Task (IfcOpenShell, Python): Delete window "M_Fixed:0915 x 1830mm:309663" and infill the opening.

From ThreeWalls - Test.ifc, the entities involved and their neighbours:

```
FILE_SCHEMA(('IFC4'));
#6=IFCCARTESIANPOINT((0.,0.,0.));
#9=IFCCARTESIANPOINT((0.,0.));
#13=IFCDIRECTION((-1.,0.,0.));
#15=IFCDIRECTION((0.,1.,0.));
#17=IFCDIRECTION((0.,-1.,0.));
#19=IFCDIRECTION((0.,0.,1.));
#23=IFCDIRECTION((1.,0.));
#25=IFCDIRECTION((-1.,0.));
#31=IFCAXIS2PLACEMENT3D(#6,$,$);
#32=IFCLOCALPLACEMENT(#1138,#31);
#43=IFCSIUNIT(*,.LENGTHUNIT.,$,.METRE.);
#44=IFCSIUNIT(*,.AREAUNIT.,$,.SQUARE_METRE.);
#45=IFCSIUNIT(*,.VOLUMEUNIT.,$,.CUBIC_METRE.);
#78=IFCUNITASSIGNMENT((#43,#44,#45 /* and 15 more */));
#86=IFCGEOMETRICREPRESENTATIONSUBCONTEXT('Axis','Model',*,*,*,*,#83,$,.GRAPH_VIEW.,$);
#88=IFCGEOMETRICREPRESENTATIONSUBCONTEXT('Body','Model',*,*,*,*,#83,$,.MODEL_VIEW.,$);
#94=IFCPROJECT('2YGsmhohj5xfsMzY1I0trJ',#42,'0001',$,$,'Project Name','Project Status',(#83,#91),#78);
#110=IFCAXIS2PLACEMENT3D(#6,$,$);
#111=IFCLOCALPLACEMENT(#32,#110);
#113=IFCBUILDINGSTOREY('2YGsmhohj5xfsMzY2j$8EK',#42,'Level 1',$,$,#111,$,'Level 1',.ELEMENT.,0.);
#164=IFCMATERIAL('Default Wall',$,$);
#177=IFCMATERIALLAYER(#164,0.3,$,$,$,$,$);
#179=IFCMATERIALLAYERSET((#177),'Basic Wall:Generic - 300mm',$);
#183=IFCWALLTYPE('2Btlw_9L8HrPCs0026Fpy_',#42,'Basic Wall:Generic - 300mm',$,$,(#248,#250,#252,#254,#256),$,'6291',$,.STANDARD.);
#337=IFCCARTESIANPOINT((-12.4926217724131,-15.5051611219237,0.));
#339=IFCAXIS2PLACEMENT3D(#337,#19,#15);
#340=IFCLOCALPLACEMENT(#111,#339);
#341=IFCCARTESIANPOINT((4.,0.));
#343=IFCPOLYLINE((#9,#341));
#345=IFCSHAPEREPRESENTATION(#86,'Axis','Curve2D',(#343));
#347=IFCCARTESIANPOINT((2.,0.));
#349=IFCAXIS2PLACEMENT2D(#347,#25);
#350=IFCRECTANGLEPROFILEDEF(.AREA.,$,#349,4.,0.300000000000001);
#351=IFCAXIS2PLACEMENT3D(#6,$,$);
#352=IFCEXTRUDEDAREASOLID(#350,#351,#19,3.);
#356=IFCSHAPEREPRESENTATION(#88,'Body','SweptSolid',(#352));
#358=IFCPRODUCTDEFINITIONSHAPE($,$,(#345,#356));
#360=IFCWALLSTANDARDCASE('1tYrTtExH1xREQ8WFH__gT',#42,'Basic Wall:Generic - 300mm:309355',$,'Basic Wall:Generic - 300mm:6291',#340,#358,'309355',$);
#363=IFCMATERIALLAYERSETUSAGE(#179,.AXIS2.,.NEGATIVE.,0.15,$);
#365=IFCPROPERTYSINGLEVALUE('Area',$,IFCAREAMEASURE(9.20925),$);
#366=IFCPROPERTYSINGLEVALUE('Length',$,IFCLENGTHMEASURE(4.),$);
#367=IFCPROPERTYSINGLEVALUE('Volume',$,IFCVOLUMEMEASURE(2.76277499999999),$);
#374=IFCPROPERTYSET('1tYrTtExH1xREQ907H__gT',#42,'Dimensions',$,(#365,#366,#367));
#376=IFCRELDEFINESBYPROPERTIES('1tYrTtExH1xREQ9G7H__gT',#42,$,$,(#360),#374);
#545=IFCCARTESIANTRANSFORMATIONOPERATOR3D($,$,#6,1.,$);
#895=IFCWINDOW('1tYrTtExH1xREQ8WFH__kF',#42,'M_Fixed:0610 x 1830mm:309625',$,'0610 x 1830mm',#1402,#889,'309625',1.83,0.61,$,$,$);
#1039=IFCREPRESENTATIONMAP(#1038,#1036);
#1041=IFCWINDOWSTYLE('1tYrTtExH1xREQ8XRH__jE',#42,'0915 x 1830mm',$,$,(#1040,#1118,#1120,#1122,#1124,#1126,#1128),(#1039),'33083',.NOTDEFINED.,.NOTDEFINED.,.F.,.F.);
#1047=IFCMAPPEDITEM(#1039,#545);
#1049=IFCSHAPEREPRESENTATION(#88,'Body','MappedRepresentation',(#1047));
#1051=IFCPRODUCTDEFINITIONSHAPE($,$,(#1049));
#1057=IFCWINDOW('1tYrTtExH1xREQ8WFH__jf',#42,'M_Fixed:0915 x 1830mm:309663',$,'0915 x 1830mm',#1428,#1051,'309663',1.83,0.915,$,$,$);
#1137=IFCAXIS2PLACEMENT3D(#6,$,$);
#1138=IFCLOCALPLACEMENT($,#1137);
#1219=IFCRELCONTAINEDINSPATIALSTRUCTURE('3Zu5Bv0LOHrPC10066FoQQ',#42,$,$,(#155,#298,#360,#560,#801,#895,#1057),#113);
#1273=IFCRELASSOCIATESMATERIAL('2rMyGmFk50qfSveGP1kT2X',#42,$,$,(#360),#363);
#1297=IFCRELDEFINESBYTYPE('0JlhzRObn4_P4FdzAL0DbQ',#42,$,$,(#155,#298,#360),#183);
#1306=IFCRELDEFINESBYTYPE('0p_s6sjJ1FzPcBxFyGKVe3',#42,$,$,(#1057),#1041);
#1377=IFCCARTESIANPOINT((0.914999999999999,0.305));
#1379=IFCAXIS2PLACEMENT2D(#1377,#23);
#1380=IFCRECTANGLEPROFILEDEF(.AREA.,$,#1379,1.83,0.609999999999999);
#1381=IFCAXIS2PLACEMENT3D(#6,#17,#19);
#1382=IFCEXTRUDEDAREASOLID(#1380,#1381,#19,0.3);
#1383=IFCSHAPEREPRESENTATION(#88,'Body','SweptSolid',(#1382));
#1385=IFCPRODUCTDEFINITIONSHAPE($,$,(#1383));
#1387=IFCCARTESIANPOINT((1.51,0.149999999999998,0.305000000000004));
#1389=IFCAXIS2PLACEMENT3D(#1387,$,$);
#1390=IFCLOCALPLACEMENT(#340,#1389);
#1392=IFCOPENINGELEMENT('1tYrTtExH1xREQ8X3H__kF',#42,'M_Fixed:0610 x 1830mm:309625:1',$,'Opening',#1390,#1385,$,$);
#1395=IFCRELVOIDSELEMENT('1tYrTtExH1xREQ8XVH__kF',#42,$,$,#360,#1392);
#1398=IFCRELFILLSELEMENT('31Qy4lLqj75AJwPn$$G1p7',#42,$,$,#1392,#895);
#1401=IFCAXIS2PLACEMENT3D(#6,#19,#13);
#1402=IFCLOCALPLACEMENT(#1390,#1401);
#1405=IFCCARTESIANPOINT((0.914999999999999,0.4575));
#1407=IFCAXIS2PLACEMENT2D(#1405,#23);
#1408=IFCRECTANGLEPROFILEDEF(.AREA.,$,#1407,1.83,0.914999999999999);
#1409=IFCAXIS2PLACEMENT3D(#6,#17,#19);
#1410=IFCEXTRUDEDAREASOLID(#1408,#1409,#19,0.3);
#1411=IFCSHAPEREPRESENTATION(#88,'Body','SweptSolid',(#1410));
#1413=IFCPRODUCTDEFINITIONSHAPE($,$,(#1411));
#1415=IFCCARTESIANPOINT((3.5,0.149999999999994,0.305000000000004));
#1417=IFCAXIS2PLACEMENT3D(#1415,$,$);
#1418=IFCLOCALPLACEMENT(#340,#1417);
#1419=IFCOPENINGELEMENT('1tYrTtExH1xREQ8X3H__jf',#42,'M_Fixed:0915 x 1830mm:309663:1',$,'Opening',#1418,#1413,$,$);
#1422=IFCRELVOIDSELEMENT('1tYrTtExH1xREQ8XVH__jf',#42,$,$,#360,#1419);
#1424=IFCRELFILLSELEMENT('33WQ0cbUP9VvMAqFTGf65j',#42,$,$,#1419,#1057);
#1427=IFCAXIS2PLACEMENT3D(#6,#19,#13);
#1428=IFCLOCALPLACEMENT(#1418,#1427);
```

```python
import ifcopenshell
import ifcopenshell.api.feature
import ifcopenshell.api.pset
import ifcopenshell.api.root
import ifcopenshell.geom
import ifcopenshell.util.element
import ifcopenshell.util.shape
import ifcopenshell.util.unit

model = ifcopenshell.open("ThreeWalls - Test.ifc")
area_scale = ifcopenshell.util.unit.calculate_unit_scale(model, "AREAUNIT")
volume_scale = ifcopenshell.util.unit.calculate_unit_scale(model, "VOLUMEUNIT")
settings = ifcopenshell.geom.settings()


def volume(element):
    """Net volume in cubic metres, openings subtracted."""
    shape = ifcopenshell.geom.create_shape(settings, element)
    return ifcopenshell.util.shape.get_volume(shape.geometry)


window = model.by_guid("1tYrTtExH1xREQ8WFH__jf")
opening = window.FillsVoids[0].RelatingOpeningElement
wall = opening.VoidsElements[0].RelatingBuildingElement
before = volume(wall)

ifcopenshell.api.root.remove_product(model, product=window)
ifcopenshell.api.feature.remove_feature(model, feature=opening)

after = volume(wall)
thickness = 0.3  # wall thickness in metres

# Update the wall's stored quantities.
pset = model.by_id(ifcopenshell.util.element.get_pset(wall, "Dimensions", should_inherit=False)["id"])
ifcopenshell.api.pset.edit_pset(model, pset=pset, properties={
    "Area": model.create_entity("IfcAreaMeasure", after / thickness / area_scale),
    "Volume": model.create_entity("IfcVolumeMeasure", after / volume_scale),
})

print(f"wall volume {before:.3f} -> {after:.3f} m3")

model.write("ThreeWalls - Test_v2.ifc")
```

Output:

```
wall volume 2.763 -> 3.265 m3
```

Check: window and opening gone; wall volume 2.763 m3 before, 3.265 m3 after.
